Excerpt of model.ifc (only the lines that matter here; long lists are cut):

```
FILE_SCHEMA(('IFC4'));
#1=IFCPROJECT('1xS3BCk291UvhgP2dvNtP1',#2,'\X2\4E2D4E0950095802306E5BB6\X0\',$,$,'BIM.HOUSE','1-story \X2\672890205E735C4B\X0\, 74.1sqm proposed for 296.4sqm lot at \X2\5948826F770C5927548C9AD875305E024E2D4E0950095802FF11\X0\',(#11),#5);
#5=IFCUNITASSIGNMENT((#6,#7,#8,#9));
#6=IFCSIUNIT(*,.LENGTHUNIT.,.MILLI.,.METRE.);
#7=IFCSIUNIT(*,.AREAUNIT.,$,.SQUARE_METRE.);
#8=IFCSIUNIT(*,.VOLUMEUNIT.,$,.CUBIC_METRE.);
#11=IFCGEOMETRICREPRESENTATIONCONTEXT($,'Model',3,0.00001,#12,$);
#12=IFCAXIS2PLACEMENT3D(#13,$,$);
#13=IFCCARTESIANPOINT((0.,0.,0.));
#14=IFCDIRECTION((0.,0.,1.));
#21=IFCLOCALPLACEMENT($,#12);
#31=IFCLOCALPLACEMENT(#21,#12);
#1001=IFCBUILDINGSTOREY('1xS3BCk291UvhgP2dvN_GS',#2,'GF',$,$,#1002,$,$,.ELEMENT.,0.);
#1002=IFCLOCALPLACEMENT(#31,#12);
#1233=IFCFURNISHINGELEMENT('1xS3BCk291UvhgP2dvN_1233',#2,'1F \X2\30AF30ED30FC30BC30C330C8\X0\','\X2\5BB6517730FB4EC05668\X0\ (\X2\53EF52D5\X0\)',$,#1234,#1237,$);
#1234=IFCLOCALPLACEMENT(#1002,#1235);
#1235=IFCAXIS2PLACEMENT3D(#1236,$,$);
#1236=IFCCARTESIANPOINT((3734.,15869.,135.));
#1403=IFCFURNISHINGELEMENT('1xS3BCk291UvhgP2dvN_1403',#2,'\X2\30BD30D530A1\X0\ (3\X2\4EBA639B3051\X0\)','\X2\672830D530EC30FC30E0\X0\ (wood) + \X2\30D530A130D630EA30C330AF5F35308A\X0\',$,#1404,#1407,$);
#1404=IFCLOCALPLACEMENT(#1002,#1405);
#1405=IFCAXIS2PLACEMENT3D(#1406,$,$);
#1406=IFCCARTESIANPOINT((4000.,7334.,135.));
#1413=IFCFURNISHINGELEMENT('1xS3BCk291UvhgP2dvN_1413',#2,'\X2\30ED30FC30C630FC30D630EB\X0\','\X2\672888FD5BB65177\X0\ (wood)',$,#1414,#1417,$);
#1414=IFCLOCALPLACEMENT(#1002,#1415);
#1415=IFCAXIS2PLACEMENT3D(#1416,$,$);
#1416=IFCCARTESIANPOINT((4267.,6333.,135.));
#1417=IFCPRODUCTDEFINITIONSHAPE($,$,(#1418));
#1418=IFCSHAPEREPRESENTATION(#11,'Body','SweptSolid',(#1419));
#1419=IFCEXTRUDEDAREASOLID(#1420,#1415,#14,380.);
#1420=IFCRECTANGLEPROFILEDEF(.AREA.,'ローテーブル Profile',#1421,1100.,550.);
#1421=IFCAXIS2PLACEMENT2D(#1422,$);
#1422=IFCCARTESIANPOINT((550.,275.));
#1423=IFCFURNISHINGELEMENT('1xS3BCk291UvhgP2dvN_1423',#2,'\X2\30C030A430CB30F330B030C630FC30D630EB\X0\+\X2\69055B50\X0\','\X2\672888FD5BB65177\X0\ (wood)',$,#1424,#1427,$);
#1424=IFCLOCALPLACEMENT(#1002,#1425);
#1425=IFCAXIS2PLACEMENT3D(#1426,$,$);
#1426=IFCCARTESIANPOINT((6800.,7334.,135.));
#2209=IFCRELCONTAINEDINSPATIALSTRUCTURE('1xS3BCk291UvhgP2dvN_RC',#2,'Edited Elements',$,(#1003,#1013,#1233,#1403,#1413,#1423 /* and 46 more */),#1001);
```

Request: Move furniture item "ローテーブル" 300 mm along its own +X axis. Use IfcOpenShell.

```python
import ifcopenshell
import ifcopenshell.api.geometry
import ifcopenshell.util.placement
import ifcopenshell.util.unit

model = ifcopenshell.open("model.ifc")
unit_scale = ifcopenshell.util.unit.calculate_unit_scale(model)

item = model.by_guid("1xS3BCk291UvhgP2dvN_1413")
matrix = ifcopenshell.util.placement.get_local_placement(item.ObjectPlacement)
matrix[:3, 3] += matrix[:3, 0] * 0.3 / unit_scale
ifcopenshell.api.geometry.edit_object_placement(model, product=item, matrix=matrix, is_si=False)

print(ifcopenshell.util.placement.get_local_placement(item.ObjectPlacement).round(3) + 0.0)

model.write("model_v2.ifc")
```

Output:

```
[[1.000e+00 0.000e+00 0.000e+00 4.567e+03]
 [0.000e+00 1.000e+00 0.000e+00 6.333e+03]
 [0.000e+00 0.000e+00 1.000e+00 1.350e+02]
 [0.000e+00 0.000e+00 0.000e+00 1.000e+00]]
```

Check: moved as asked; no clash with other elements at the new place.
